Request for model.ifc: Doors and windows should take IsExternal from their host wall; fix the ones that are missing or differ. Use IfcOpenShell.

First a look at what the model holds.

```python
import ifcopenshell
import ifcopenshell.util.element

model = ifcopenshell.open("model.ifc")
print(model.schema)
seen = {}
for e in model.by_type("IfcDoor") + model.by_type("IfcWindow"):
    if not e.FillsVoids:
        continue
    host = e.FillsVoids[0].RelatingOpeningElement.VoidsElements[0].RelatingBuildingElement
    own = ifcopenshell.util.element.get_pset(e, f"Pset_{e.is_a()[3:].removesuffix('StandardCase')}Common", "IsExternal")
    wall = ifcopenshell.util.element.get_pset(host, "Pset_WallCommon", "IsExternal")
    seen[e.is_a(), own, wall] = seen.get((e.is_a(), own, wall), 0) + 1
for (cls, own, wall), count in sorted(seen.items(), key=str):
    print(count, cls, "IsExternal:", own, "| host wall:", wall)
```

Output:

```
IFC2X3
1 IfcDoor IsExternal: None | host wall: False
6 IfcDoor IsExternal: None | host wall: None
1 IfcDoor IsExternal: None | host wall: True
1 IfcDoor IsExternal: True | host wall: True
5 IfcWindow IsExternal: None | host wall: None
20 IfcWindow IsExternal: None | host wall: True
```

```python
import ifcopenshell
import ifcopenshell.api.pset
import ifcopenshell.util.element

model = ifcopenshell.open("model.ifc")

count = 0
for ifc_class, pset_name in (("IfcDoor", "Pset_DoorCommon"), ("IfcWindow", "Pset_WindowCommon")):
    for e in model.by_type(ifc_class):
        if not e.FillsVoids:
            continue
        host = e.FillsVoids[0].RelatingOpeningElement.VoidsElements[0].RelatingBuildingElement
        external = ifcopenshell.util.element.get_pset(host, "Pset_WallCommon", "IsExternal")
        if external is None or ifcopenshell.util.element.get_pset(e, pset_name, "IsExternal") == external:
            continue
        pset = ifcopenshell.api.pset.add_pset(model, product=e, name=pset_name)
        ifcopenshell.api.pset.edit_pset(model, pset=pset, properties={"IsExternal": external})
        count += 1

print(count, "updated")

model.write("model_v2.ifc")
```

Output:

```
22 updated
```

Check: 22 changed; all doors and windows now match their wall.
